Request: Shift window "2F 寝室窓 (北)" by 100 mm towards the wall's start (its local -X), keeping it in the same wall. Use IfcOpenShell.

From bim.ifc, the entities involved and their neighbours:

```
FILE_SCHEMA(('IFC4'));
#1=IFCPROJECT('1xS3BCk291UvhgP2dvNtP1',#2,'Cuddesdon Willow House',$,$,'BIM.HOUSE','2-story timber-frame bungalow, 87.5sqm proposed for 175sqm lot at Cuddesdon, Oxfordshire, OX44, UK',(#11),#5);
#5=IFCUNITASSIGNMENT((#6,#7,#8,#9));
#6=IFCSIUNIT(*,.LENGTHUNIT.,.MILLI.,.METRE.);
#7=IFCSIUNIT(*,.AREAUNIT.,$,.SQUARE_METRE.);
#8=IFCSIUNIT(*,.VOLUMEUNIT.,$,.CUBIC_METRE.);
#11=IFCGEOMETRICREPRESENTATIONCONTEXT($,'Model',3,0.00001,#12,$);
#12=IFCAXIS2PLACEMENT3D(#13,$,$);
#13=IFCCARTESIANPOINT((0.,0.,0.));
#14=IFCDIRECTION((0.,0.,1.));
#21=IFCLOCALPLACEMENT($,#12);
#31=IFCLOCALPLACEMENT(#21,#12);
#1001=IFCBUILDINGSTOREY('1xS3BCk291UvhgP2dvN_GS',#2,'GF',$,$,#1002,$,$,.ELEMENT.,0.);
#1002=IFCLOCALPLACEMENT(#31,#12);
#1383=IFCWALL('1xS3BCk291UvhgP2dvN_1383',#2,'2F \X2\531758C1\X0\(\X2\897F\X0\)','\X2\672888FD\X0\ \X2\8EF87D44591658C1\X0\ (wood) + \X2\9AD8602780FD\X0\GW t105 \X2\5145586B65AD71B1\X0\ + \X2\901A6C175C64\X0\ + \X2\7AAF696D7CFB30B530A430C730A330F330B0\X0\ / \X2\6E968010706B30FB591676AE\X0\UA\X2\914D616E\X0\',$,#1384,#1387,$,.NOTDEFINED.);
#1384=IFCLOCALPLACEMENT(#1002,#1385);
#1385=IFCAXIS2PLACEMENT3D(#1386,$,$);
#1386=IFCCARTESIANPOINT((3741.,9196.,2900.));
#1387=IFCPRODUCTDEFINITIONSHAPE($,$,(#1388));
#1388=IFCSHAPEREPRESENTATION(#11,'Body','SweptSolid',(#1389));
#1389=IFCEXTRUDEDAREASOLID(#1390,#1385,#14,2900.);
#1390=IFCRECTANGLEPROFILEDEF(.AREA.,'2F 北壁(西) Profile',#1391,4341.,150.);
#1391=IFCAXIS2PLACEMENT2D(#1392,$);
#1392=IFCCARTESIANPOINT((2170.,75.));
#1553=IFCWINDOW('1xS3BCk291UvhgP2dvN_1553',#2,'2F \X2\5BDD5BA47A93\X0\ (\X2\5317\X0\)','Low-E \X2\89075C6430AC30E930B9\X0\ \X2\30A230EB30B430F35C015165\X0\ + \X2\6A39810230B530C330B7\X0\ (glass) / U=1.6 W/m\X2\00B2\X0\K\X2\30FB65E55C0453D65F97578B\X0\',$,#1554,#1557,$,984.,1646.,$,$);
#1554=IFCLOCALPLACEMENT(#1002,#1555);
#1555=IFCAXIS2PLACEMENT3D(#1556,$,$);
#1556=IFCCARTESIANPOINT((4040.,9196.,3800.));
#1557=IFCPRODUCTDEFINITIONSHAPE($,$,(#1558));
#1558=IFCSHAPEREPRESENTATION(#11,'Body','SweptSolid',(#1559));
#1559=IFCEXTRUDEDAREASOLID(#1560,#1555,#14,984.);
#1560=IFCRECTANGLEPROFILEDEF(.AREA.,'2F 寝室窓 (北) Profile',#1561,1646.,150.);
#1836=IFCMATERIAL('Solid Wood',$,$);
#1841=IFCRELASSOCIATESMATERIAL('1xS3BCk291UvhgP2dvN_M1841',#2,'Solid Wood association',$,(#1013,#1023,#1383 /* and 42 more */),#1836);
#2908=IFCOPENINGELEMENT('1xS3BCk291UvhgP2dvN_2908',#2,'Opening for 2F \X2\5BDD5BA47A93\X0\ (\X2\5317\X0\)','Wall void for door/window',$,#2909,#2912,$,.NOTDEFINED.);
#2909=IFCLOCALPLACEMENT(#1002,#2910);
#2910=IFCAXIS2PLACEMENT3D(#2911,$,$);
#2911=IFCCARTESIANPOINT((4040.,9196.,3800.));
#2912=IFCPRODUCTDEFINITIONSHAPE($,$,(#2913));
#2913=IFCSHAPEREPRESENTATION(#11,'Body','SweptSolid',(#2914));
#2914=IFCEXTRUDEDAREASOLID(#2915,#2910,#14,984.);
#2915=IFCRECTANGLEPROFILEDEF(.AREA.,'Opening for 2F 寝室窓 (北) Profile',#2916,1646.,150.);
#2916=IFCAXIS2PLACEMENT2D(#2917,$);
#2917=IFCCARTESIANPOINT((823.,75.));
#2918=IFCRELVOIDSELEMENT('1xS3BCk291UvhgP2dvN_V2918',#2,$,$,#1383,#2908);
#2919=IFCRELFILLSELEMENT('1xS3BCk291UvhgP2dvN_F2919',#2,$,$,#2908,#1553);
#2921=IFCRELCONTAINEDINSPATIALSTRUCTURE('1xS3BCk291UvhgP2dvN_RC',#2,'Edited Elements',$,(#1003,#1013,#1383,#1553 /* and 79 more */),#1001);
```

```python
import ifcopenshell
import ifcopenshell.api.geometry
import ifcopenshell.util.placement

model = ifcopenshell.open("bim.ifc")

window = model.by_id(1553)
opening = window.FillsVoids[0].RelatingOpeningElement
wall = opening.VoidsElements[0].RelatingBuildingElement

wall_matrix = ifcopenshell.util.placement.get_local_placement(wall.ObjectPlacement)
shift = wall_matrix[:3, 0] * -100.0
before = ifcopenshell.util.placement.get_local_placement(window.ObjectPlacement)[:3, 3].copy()

# The window is not placed relative to its opening, so move both.
for product in (opening, window):
    matrix = ifcopenshell.util.placement.get_local_placement(product.ObjectPlacement)
    matrix[:3, 3] += shift
    ifcopenshell.api.geometry.edit_object_placement(model, product=product, matrix=matrix, is_si=False)

after = ifcopenshell.util.placement.get_local_placement(window.ObjectPlacement)[:3, 3]
print("window moved by", (after - before).round(3) + 0.0)

model.write("bim_edited.ifc")
```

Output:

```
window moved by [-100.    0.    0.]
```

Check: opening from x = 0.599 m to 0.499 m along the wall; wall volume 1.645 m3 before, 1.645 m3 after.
